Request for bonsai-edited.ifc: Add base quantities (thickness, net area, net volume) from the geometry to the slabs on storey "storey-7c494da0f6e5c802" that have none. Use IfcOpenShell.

First a look at what the model holds.

```python
import ifcopenshell
import ifcopenshell.util.element
import ifcopenshell.util.unit

model = ifcopenshell.open("bonsai-edited.ifc")
print(model.schema)
for unit_type in ("LENGTHUNIT", "AREAUNIT", "VOLUMEUNIT"):
    print(unit_type, ifcopenshell.util.unit.calculate_unit_scale(model, unit_type))
storey = next(s for s in model.by_type("IfcBuildingStorey") if s.Name == "storey-7c494da0f6e5c802")
slabs = [e for e in ifcopenshell.util.element.get_decomposition(storey) if e.is_a("IfcSlab")]
for e in sorted(slabs, key=lambda e: e.id()):
    print(e.id(), e.is_a(), e.Name, list(ifcopenshell.util.element.get_psets(e, qtos_only=True)), sep=" | ")
```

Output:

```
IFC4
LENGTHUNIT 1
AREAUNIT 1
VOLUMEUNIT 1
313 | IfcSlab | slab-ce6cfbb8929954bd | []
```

```python
import ifcopenshell
import ifcopenshell.api.pset
import ifcopenshell.geom
import ifcopenshell.util.element
import ifcopenshell.util.shape
import ifcopenshell.util.unit

model = ifcopenshell.open("bonsai-edited.ifc")
unit_scale = ifcopenshell.util.unit.calculate_unit_scale(model)
area_scale = ifcopenshell.util.unit.calculate_unit_scale(model, "AREAUNIT")
volume_scale = ifcopenshell.util.unit.calculate_unit_scale(model, "VOLUMEUNIT")
settings = ifcopenshell.geom.settings()

storey = next(s for s in model.by_type("IfcBuildingStorey") if s.Name == "storey-7c494da0f6e5c802")
slabs = [e for e in ifcopenshell.util.element.get_decomposition(storey) if e.is_a("IfcSlab")]

for e in sorted(slabs, key=lambda e: e.id()):
    if ifcopenshell.util.element.get_psets(e, qtos_only=True, should_inherit=False):
        continue
    # Geometry comes back in metres, in the element's own axes.
    shape = ifcopenshell.geom.create_shape(settings, e)
    values = {
        "Width": ifcopenshell.util.shape.get_z(shape.geometry) / unit_scale,
        "NetArea": ifcopenshell.util.shape.get_footprint_area(shape.geometry) / area_scale,
        "NetVolume": ifcopenshell.util.shape.get_volume(shape.geometry) / volume_scale,
    }
    qto = ifcopenshell.api.pset.add_qto(model, product=e, name="Qto_SlabBaseQuantities")
    ifcopenshell.api.pset.edit_qto(model, qto=qto, properties=values)
    print(e.id(), {k: round(v, 3) for k, v in values.items()})

model.write("bonsai-edited_rev.ifc")
```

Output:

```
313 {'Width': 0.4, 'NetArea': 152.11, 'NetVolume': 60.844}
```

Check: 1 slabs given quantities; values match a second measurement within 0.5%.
